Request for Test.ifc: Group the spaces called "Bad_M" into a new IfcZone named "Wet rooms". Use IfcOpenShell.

First a look at what the model holds.

```python
import ifcopenshell

model = ifcopenshell.open("Test.ifc")
print(model.schema)
seen = {}
for space in model.by_type("IfcSpace"):
    seen[space.LongName] = seen.get(space.LongName, 0) + 1
for name, count in sorted(seen.items(), key=str):
    print(count, "x", name)
print("zones:", [z.Name for z in model.by_type("IfcZone")][:20])
```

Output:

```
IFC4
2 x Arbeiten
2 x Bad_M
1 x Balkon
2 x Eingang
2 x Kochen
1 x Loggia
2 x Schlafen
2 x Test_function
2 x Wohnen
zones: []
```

```python
import ifcopenshell
import ifcopenshell.api.group
import ifcopenshell.api.root

model = ifcopenshell.open("Test.ifc")

names = {"Bad_M"}
spaces = [s for s in model.by_type("IfcSpace") if s.LongName in names]

zone = ifcopenshell.api.root.create_entity(model, ifc_class="IfcZone", name="Wet rooms")
ifcopenshell.api.group.assign_group(model, products=spaces, group=zone)
print(len(spaces), "spaces in", zone.Name)

model.write("Test-out.ifc")
```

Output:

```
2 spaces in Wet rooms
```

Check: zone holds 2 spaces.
